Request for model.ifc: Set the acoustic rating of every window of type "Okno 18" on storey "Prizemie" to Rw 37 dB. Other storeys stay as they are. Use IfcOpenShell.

First a look at what the model holds.

```python
import ifcopenshell
import ifcopenshell.util.element

model = ifcopenshell.open("model.ifc")
print(model.schema)
storey = next(s for s in model.by_type("IfcBuildingStorey") if s.Name == "Prizemie")
windows = [e for e in ifcopenshell.util.element.get_decomposition(storey) if e.is_a("IfcWindow")]
seen = {}
for e in windows:
    element_type = ifcopenshell.util.element.get_type(e)
    key = (element_type.Name if element_type != e and element_type else None, ifcopenshell.util.element.get_pset(e, "Pset_WindowCommon", "AcousticRating"))
    seen[key] = seen.get(key, 0) + 1
for (name, value), count in sorted(seen.items(), key=str):
    print(count, "x", name, "|", value)
```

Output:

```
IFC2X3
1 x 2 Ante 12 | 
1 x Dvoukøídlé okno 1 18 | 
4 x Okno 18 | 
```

```python
import ifcopenshell
import ifcopenshell.api.pset
import ifcopenshell.util.element

model = ifcopenshell.open("model.ifc")

storey = next(s for s in model.by_type("IfcBuildingStorey") if s.Name == "Prizemie")
windows = [e for e in ifcopenshell.util.element.get_decomposition(storey) if e.is_a("IfcWindow")]

count = 0
for e in windows:
    element_type = ifcopenshell.util.element.get_type(e)
    if element_type in (None, e) or element_type.Name != "Okno 18":
        continue
    # add_pset returns the element's existing set when there is one.
    pset = ifcopenshell.api.pset.add_pset(model, product=e, name="Pset_WindowCommon")
    ifcopenshell.api.pset.edit_pset(model, pset=pset, properties={"AcousticRating": "Rw 37 dB"})
    count += 1

print(count, "windows updated")

model.write("model-out.ifc")
```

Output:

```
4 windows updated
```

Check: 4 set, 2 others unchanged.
